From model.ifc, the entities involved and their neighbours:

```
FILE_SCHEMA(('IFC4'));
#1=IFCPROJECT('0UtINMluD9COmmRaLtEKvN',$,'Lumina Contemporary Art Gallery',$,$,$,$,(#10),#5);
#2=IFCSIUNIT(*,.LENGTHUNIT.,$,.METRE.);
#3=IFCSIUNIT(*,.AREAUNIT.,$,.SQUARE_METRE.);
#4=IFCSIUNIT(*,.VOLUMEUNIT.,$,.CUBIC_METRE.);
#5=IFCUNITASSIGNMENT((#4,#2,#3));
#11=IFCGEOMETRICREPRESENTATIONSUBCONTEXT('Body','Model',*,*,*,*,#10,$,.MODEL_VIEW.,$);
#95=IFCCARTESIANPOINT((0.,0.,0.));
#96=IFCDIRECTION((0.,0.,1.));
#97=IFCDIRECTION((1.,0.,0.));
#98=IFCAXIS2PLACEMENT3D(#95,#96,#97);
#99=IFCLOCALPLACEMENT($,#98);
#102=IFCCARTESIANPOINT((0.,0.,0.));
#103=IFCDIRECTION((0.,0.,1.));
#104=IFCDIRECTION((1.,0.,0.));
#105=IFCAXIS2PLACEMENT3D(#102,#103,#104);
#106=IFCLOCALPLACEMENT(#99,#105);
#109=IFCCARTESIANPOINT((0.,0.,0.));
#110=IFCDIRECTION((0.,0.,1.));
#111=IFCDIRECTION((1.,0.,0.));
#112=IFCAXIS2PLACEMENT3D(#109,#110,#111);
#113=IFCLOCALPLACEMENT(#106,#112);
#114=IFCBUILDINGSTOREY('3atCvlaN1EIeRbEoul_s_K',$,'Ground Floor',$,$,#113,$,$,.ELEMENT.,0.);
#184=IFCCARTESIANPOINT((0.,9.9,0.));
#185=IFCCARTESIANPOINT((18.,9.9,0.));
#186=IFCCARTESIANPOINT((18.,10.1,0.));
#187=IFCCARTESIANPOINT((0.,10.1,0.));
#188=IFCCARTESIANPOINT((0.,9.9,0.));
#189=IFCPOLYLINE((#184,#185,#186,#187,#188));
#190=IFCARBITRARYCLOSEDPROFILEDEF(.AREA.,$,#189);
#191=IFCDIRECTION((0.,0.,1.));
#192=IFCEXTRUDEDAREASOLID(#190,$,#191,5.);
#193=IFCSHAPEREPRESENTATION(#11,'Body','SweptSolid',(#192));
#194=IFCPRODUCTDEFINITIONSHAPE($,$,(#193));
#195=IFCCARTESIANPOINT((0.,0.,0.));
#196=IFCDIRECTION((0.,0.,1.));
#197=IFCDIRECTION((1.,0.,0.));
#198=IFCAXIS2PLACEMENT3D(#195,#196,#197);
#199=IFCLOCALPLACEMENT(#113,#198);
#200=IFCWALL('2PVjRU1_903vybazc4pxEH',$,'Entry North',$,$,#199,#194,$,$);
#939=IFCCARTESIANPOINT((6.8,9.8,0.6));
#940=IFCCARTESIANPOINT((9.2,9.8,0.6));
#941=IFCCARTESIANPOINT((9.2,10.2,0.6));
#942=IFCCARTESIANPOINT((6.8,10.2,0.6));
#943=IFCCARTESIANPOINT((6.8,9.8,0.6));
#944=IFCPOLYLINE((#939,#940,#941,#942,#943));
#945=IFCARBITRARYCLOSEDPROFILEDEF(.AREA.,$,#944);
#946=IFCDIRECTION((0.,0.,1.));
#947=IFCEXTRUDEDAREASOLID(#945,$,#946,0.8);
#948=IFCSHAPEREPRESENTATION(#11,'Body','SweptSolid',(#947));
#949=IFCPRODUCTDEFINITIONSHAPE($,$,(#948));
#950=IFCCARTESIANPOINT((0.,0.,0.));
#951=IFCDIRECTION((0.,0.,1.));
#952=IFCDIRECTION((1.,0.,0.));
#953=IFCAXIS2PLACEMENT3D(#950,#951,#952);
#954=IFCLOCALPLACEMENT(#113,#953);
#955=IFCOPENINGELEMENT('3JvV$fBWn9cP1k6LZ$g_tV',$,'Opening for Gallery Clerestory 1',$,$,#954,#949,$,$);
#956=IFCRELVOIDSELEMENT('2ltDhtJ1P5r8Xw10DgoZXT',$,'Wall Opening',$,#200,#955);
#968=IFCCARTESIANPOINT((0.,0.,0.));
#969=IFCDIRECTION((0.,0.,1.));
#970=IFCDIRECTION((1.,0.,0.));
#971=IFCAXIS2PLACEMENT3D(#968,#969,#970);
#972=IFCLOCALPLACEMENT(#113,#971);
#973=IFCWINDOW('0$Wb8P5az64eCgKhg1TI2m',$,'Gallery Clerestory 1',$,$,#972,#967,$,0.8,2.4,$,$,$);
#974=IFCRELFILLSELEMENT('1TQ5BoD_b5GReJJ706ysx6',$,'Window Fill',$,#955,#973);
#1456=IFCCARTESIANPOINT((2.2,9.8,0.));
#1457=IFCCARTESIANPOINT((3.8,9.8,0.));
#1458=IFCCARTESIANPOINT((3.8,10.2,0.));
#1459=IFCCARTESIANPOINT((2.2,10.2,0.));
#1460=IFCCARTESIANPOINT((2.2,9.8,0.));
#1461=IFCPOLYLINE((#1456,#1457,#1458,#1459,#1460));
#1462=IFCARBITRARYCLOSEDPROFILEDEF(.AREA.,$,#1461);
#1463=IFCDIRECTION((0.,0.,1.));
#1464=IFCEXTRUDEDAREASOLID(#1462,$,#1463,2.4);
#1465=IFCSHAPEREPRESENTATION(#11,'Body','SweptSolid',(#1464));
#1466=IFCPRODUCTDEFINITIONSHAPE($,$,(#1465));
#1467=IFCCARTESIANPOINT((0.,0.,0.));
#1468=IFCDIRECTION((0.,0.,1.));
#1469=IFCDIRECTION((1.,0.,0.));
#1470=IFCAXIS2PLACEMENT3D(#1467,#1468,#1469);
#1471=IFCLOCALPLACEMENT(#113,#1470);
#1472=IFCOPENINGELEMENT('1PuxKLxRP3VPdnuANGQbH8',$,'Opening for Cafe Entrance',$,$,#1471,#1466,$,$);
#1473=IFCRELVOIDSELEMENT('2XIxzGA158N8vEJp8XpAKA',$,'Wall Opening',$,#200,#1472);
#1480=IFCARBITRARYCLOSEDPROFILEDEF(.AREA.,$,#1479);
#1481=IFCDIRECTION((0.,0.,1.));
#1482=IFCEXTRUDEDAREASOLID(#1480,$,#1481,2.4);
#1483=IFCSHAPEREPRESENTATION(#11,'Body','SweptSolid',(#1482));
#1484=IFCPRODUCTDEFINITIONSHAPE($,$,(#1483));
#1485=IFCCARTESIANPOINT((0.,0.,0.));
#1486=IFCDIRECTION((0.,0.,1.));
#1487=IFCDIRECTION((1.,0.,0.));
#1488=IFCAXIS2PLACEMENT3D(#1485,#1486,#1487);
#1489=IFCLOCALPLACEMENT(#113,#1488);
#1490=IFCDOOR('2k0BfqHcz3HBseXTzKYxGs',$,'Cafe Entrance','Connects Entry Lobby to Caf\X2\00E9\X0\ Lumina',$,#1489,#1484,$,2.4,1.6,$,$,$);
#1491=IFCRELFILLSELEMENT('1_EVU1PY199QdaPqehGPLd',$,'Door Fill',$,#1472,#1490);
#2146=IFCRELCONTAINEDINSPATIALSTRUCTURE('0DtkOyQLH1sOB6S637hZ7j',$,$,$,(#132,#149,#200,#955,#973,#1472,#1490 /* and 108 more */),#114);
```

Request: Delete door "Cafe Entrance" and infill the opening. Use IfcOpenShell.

```python
import ifcopenshell
import ifcopenshell.api.feature
import ifcopenshell.api.root
import ifcopenshell.geom
import ifcopenshell.util.shape

model = ifcopenshell.open("model.ifc")
settings = ifcopenshell.geom.settings()


def volume(element):
    """Net volume in cubic metres, openings subtracted."""
    shape = ifcopenshell.geom.create_shape(settings, element)
    return ifcopenshell.util.shape.get_volume(shape.geometry)


door = model.by_id(1490)
opening = door.FillsVoids[0].RelatingOpeningElement
wall = opening.VoidsElements[0].RelatingBuildingElement
before = volume(wall)

ifcopenshell.api.root.remove_product(model, product=door)
ifcopenshell.api.feature.remove_feature(model, feature=opening)

after = volume(wall)

print(f"wall volume {before:.3f} -> {after:.3f} m3")

model.write("model_rev.ifc")
```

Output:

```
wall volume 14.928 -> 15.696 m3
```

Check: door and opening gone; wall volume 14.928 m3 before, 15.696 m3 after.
